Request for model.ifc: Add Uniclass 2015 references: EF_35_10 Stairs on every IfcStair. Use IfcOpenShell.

First a look at what the model holds.

```python
import ifcopenshell

model = ifcopenshell.open("model.ifc")
print(model.schema)
print("classifications:", [c.Name for c in model.by_type("IfcClassification")])
for ifc_class in ("IfcDoor", "IfcRoof", "IfcStair", "IfcWall", "IfcWindow"):
    print(ifc_class, len(model.by_type(ifc_class)))
```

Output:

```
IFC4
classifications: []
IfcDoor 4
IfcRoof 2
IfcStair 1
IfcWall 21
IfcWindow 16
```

```python
import ifcopenshell
import ifcopenshell.api.classification

model = ifcopenshell.open("model.ifc")

system = ifcopenshell.api.classification.add_classification(model, classification="Uniclass 2015")

codes = {
    "IfcStair": ("EF_35_10", "Stairs"),
}
for ifc_class, (code, name) in codes.items():
    products = model.by_type(ifc_class)
    ifcopenshell.api.classification.add_reference(
        model, products=products, classification=system, identification=code, name=name
    )
    print(code, len(products))

model.write("model_edited.ifc")
```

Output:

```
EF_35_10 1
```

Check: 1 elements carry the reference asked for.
